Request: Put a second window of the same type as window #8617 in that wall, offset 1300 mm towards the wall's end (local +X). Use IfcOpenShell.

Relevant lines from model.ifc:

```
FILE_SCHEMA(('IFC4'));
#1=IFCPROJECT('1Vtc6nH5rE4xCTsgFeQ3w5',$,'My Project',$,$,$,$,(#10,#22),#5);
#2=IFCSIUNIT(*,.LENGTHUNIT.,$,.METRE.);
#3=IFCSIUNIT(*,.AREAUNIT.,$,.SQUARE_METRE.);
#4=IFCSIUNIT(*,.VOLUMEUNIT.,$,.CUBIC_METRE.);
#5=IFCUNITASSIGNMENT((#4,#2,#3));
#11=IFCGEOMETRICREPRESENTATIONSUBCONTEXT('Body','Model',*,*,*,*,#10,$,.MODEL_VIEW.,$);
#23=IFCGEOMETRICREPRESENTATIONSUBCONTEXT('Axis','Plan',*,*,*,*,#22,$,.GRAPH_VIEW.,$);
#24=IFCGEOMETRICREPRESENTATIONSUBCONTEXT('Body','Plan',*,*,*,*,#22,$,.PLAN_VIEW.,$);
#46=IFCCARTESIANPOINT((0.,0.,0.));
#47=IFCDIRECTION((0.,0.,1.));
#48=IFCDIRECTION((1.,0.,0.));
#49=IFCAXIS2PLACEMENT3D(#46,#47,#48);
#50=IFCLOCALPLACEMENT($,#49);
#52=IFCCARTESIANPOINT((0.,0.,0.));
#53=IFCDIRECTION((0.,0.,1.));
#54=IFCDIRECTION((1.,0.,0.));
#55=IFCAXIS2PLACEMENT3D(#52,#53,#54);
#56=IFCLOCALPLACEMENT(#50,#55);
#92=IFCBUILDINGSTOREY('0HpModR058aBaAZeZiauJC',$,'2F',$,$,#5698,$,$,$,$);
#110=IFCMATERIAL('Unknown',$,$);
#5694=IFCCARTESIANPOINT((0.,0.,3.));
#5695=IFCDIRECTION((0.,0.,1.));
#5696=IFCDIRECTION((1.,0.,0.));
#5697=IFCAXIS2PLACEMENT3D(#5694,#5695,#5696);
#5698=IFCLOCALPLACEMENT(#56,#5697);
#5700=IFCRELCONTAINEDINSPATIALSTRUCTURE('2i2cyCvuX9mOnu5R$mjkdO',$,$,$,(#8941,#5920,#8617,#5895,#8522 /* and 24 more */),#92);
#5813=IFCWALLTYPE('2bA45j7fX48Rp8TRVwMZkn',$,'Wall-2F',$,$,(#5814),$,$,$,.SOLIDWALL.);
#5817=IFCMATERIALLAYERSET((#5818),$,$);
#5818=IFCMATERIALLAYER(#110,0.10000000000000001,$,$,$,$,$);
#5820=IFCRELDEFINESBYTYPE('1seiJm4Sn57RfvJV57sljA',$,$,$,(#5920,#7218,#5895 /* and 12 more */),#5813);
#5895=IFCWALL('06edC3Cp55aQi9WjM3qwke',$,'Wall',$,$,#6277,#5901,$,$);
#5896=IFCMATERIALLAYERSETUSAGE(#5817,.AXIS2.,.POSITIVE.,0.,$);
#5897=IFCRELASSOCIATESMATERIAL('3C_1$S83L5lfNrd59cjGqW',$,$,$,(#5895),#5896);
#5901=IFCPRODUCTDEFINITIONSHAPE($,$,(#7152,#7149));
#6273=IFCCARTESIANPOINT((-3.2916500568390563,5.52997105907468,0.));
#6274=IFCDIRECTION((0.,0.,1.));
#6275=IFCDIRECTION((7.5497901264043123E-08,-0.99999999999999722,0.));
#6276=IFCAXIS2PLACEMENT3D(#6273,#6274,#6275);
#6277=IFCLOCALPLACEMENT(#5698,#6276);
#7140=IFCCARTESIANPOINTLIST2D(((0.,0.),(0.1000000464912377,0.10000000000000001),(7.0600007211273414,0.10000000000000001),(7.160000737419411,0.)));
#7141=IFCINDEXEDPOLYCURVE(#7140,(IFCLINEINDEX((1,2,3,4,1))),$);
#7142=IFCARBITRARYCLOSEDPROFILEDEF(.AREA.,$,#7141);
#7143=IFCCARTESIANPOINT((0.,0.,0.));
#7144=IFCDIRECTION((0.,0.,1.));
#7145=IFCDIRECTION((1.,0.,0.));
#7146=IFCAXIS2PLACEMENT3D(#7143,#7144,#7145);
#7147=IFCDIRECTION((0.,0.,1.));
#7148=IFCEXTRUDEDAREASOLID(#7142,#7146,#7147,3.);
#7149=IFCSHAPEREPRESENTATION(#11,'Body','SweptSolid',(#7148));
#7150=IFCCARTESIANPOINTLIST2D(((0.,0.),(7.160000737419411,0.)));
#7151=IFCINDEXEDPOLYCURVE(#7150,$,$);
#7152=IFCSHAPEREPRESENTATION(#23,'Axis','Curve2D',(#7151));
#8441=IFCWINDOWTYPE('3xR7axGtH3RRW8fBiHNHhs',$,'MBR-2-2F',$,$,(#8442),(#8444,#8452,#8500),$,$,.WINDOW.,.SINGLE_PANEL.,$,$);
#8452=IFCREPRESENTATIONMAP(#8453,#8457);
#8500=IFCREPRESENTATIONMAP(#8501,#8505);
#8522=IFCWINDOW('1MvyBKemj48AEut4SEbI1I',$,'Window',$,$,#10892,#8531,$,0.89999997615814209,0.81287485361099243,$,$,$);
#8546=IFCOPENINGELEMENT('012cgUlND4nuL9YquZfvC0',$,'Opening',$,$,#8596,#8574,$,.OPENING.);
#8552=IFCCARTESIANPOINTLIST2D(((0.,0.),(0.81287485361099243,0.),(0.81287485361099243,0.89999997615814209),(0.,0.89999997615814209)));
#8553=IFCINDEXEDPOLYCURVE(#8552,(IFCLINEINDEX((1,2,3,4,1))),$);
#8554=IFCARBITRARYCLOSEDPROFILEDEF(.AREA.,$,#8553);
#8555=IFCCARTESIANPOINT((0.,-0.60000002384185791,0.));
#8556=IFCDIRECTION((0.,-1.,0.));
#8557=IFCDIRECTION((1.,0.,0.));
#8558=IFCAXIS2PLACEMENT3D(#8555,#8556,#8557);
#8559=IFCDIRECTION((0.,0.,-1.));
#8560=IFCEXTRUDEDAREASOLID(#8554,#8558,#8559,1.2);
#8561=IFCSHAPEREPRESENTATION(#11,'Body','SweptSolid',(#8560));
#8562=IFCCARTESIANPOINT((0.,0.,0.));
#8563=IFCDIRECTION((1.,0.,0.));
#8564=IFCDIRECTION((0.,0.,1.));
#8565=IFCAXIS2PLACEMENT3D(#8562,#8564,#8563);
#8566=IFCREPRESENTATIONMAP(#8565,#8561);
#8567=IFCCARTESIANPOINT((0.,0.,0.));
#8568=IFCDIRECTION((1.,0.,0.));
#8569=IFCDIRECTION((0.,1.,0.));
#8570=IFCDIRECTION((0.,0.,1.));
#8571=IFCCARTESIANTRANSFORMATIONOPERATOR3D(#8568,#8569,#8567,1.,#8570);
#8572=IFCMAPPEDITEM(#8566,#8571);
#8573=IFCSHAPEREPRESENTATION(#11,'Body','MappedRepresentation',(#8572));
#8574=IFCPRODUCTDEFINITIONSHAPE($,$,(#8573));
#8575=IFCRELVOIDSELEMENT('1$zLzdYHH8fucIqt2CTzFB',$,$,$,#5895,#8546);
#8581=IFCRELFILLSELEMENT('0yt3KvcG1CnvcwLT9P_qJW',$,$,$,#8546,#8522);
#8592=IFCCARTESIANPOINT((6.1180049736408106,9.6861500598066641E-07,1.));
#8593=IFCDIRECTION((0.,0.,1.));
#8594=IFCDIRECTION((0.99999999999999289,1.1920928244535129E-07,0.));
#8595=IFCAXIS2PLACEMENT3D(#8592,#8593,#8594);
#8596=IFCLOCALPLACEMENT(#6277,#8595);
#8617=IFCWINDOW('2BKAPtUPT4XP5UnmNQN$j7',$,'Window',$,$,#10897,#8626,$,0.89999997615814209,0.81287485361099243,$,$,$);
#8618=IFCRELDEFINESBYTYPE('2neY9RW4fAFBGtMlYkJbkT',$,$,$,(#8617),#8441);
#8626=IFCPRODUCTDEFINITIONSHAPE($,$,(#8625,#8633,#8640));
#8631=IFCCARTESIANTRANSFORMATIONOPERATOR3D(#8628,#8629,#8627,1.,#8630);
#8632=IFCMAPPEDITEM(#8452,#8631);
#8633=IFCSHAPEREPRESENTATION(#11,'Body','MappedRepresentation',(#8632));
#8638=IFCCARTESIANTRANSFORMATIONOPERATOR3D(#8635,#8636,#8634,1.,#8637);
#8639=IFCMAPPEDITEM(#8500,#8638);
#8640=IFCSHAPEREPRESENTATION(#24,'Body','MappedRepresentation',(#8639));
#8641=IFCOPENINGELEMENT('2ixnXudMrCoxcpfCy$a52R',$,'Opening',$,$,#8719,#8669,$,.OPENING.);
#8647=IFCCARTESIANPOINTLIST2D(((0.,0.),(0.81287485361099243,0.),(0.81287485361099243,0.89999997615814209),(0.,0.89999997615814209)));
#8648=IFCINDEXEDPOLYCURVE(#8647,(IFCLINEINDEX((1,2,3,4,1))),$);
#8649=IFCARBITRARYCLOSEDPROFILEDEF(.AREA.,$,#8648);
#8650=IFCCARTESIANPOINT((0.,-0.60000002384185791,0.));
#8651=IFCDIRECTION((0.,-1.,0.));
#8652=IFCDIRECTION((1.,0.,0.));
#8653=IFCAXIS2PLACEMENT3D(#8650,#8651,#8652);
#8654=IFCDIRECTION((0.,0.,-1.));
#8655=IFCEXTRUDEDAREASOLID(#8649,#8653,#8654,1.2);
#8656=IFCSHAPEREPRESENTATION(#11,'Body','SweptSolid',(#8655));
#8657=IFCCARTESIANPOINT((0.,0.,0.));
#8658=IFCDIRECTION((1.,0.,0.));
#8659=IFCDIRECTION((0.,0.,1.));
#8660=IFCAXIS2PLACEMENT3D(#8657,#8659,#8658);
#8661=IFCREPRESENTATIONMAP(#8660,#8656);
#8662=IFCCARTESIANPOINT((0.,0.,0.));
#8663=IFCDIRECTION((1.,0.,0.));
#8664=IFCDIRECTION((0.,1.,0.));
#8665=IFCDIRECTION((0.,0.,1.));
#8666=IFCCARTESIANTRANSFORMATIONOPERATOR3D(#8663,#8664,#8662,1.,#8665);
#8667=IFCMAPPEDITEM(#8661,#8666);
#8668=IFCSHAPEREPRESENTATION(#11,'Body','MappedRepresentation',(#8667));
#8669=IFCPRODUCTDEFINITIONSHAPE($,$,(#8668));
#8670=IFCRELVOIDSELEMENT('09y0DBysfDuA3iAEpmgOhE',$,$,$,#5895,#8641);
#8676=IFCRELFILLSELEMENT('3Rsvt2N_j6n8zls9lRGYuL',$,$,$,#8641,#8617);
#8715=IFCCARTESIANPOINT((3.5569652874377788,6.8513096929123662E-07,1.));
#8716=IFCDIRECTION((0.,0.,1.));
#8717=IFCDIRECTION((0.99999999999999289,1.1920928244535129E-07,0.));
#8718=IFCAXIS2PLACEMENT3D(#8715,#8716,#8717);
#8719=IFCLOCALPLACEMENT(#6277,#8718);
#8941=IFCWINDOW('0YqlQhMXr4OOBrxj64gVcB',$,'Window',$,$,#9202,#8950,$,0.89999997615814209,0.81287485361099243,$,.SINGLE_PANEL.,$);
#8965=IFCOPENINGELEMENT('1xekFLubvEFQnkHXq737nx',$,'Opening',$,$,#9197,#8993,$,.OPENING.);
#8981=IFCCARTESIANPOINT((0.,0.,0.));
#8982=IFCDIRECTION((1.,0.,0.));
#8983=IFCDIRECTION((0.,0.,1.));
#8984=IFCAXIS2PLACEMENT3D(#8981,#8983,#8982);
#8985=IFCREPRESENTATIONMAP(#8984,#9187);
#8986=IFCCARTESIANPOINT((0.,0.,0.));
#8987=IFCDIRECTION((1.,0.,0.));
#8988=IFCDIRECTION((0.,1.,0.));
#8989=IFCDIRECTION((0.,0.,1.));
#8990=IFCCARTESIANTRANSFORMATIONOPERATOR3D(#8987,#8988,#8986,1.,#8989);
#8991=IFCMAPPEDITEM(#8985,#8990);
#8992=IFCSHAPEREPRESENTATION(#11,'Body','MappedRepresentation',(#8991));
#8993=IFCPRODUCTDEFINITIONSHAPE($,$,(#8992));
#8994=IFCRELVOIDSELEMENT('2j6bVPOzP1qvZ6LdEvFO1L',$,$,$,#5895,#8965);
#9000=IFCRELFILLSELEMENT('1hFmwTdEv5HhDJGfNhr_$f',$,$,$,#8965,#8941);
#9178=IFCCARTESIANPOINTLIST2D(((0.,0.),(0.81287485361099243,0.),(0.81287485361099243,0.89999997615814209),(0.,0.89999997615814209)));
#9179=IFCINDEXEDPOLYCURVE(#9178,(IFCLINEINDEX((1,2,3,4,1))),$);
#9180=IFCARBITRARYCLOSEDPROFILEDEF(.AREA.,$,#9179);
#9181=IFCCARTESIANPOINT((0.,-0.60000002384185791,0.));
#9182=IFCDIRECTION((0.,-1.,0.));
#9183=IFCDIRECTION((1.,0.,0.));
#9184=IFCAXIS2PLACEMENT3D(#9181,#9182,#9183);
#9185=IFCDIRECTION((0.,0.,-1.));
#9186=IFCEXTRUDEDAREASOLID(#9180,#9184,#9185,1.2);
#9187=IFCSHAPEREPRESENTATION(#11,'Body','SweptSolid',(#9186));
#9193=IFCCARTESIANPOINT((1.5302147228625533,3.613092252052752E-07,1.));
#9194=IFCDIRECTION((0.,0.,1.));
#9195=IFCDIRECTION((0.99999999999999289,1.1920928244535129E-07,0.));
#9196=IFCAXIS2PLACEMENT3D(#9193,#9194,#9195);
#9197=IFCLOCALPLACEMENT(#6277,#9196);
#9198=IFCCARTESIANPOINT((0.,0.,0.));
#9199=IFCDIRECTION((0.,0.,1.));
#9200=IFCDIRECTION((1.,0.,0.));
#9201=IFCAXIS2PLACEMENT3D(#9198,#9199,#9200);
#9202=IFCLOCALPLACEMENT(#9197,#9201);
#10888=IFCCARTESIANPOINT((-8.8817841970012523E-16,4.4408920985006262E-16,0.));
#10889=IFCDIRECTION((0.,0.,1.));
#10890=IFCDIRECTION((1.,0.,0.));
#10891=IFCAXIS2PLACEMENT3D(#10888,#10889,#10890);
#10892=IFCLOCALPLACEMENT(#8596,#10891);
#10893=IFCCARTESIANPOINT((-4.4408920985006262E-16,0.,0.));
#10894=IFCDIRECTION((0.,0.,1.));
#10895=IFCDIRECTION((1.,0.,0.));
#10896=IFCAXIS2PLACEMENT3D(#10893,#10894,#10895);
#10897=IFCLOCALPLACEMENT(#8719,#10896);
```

```python
import ifcopenshell
import ifcopenshell.api.feature
import ifcopenshell.api.geometry
import ifcopenshell.api.root
import ifcopenshell.geom
import ifcopenshell.util.element
import ifcopenshell.util.placement
import ifcopenshell.util.shape

model = ifcopenshell.open("model.ifc")
settings = ifcopenshell.geom.settings()


def volume(element):
    """Net volume in cubic metres, openings subtracted."""
    shape = ifcopenshell.geom.create_shape(settings, element)
    return ifcopenshell.util.shape.get_volume(shape.geometry)


window = model.by_id(8617)
opening = window.FillsVoids[0].RelatingOpeningElement
wall = opening.VoidsElements[0].RelatingBuildingElement
before = volume(wall)
shift = ifcopenshell.util.placement.get_local_placement(wall.ObjectPlacement)[:3, 0] * 1.3

# copy_class copies the void relationship, type, container and properties, but no geometry.
new_opening = ifcopenshell.api.root.copy_class(model, product=opening)
new_opening.Representation = ifcopenshell.util.element.copy_deep(
    model, opening.Representation, exclude=["IfcGeometricRepresentationContext", "IfcRepresentationMap"]
)
new_window = ifcopenshell.api.root.copy_class(model, product=window)
new_window.Representation = ifcopenshell.util.element.copy_deep(
    model, window.Representation, exclude=["IfcGeometricRepresentationContext", "IfcRepresentationMap"]
)
ifcopenshell.api.feature.add_filling(model, opening=new_opening, element=new_window)

for old, new in ((opening, new_opening), (window, new_window)):
    matrix = ifcopenshell.util.placement.get_local_placement(old.ObjectPlacement)
    matrix[:3, 3] += shift
    ifcopenshell.api.geometry.edit_object_placement(model, product=new, matrix=matrix, is_si=False)

after = volume(wall)

print(f"wall volume {before:.3f} -> {after:.3f} m3")

model.write("model_v2.ifc")
```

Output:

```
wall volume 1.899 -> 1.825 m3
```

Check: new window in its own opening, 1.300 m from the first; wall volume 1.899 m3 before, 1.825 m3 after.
